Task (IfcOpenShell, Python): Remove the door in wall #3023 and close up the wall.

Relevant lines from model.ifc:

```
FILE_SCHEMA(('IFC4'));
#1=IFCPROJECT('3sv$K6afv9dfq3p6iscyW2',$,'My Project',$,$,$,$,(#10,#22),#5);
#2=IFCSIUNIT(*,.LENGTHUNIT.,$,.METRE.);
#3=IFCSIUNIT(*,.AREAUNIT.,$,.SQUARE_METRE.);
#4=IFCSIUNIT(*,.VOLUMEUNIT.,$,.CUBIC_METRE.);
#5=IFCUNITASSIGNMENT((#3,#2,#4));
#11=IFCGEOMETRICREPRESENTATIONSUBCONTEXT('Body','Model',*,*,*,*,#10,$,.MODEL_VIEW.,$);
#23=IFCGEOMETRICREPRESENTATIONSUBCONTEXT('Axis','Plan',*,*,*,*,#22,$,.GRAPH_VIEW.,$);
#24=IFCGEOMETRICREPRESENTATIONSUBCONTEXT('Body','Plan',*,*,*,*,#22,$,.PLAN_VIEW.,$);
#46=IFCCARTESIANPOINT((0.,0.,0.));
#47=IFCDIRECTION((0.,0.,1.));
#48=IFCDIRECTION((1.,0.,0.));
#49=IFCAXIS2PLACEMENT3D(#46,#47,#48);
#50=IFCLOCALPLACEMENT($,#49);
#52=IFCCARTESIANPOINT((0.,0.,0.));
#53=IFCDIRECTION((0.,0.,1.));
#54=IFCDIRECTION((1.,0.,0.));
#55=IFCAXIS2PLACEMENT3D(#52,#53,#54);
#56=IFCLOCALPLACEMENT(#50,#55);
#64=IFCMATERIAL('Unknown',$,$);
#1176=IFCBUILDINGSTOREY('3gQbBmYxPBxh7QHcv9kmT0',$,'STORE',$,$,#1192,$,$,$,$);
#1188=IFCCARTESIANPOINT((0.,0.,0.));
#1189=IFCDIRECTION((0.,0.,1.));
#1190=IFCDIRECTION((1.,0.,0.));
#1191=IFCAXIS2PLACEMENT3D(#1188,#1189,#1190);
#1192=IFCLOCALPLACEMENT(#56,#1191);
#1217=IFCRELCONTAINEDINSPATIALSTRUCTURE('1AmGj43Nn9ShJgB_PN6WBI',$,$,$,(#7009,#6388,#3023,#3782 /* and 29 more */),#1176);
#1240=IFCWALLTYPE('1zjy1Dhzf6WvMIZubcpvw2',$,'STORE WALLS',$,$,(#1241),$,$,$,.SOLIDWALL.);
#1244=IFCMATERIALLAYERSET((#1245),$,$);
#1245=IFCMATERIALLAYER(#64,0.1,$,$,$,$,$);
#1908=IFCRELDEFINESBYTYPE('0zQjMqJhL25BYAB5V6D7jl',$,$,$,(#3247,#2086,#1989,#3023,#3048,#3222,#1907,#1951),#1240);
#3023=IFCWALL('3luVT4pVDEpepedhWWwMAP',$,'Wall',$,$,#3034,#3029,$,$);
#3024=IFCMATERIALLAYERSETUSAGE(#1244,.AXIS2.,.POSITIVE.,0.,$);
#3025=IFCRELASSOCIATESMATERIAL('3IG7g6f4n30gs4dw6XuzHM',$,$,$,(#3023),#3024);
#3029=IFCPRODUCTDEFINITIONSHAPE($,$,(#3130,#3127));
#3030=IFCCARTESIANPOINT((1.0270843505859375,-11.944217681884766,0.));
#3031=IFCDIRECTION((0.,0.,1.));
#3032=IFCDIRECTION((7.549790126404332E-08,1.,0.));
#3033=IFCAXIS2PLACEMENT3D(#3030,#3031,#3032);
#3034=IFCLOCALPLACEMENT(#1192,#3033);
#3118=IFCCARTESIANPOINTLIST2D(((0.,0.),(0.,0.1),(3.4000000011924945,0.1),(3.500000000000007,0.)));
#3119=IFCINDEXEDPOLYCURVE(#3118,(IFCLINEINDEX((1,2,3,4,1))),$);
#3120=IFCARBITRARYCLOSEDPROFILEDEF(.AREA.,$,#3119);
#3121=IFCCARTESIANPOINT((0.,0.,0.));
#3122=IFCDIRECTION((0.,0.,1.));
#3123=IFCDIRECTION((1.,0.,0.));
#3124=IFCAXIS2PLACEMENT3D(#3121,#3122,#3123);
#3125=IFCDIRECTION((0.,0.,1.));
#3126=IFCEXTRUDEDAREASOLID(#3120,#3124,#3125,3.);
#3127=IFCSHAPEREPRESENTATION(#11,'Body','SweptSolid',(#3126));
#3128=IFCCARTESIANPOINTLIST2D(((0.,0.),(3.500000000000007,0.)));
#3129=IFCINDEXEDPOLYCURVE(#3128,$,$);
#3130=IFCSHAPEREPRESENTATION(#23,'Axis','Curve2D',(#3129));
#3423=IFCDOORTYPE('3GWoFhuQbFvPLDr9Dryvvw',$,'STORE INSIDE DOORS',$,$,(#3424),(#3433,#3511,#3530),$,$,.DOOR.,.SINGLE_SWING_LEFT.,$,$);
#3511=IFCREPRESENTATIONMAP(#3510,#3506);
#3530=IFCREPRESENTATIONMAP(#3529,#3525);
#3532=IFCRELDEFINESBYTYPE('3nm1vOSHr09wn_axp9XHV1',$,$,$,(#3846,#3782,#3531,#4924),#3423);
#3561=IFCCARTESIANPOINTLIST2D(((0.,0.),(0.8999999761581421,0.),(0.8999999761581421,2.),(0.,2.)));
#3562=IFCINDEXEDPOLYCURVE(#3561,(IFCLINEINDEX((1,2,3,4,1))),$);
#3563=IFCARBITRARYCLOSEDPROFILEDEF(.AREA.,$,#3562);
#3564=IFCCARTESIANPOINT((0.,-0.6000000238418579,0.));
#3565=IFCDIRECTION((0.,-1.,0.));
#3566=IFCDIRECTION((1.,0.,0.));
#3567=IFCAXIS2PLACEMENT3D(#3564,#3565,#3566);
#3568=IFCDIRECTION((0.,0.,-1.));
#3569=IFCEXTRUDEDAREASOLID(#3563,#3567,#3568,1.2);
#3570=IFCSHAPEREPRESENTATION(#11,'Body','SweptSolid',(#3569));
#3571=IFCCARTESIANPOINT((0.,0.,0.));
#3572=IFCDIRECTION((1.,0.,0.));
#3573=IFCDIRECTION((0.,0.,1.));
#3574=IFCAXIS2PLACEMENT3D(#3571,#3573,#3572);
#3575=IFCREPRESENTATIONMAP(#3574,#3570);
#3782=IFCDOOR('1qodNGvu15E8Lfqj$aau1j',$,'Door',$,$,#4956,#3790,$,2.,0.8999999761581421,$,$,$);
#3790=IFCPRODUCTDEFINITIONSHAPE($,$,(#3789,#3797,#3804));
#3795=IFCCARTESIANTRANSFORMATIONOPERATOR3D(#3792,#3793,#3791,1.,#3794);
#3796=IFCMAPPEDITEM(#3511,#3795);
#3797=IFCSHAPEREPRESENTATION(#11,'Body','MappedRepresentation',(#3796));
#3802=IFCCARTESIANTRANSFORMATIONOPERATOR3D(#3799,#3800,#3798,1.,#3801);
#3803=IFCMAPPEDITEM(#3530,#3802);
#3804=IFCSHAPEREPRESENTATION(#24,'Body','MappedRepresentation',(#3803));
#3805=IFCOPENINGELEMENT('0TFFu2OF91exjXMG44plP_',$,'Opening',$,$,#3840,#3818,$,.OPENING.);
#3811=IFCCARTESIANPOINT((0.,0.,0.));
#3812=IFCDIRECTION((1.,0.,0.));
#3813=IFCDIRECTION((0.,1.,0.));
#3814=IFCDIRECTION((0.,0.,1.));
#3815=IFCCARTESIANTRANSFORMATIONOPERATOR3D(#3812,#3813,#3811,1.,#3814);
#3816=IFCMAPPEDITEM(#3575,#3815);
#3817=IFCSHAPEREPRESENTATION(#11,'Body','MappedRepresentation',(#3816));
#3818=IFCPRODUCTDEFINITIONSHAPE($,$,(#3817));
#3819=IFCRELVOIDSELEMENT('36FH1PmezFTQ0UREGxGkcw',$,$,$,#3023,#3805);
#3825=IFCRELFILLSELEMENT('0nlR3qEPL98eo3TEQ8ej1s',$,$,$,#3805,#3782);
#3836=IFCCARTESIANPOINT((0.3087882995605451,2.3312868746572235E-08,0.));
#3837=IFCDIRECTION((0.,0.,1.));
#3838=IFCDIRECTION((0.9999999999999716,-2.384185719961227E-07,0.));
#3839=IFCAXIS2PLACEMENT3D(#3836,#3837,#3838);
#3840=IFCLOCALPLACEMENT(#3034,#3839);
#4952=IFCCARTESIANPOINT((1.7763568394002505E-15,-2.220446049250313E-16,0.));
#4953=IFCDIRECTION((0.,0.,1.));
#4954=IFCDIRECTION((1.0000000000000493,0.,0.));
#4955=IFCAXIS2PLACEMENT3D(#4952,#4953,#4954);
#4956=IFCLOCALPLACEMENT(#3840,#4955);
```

```python
import ifcopenshell
import ifcopenshell.api.feature
import ifcopenshell.api.root
import ifcopenshell.geom
import ifcopenshell.util.shape

model = ifcopenshell.open("model.ifc")
settings = ifcopenshell.geom.settings()


def volume(element):
    """Net volume in cubic metres, openings subtracted."""
    shape = ifcopenshell.geom.create_shape(settings, element)
    return ifcopenshell.util.shape.get_volume(shape.geometry)


door = model.by_id(3782)
opening = door.FillsVoids[0].RelatingOpeningElement
wall = opening.VoidsElements[0].RelatingBuildingElement
before = volume(wall)

ifcopenshell.api.root.remove_product(model, product=door)
ifcopenshell.api.feature.remove_feature(model, feature=opening)

after = volume(wall)

print(f"wall volume {before:.3f} -> {after:.3f} m3")

model.write("model_updated.ifc")
```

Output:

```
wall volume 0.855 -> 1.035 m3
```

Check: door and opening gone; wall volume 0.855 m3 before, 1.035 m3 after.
